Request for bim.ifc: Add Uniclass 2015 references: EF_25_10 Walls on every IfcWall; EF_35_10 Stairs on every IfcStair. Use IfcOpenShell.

First a look at what the model holds.

```python
import ifcopenshell

model = ifcopenshell.open("bim.ifc")
print(model.schema)
print("classifications:", [c.Name for c in model.by_type("IfcClassification")])
for ifc_class in ("IfcDoor", "IfcRoof", "IfcStair", "IfcWall", "IfcWindow"):
    print(ifc_class, len(model.by_type(ifc_class)))
```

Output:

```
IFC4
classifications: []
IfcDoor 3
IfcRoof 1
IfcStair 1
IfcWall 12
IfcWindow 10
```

```python
import ifcopenshell
import ifcopenshell.api.classification

model = ifcopenshell.open("bim.ifc")

system = ifcopenshell.api.classification.add_classification(model, classification="Uniclass 2015")

codes = {
    "IfcWall": ("EF_25_10", "Walls"),
    "IfcStair": ("EF_35_10", "Stairs"),
}
for ifc_class, (code, name) in codes.items():
    products = model.by_type(ifc_class)
    ifcopenshell.api.classification.add_reference(
        model, products=products, classification=system, identification=code, name=name
    )
    print(code, len(products))

model.write("bim-out.ifc")
```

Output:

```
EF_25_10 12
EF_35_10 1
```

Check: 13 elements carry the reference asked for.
